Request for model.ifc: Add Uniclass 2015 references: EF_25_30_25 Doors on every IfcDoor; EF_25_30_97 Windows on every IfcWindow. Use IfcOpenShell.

First a look at what the model holds.

```python
import ifcopenshell

model = ifcopenshell.open("model.ifc")
print(model.schema)
print("classifications:", [c.Name for c in model.by_type("IfcClassification")])
for ifc_class in ("IfcDoor", "IfcRoof", "IfcStair", "IfcWall", "IfcWindow"):
    print(ifc_class, len(model.by_type(ifc_class)))
```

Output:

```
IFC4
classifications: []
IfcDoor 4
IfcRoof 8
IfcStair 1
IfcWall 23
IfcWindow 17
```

```python
import ifcopenshell
import ifcopenshell.api.classification

model = ifcopenshell.open("model.ifc")

system = ifcopenshell.api.classification.add_classification(model, classification="Uniclass 2015")

codes = {
    "IfcDoor": ("EF_25_30_25", "Doors"),
    "IfcWindow": ("EF_25_30_97", "Windows"),
}
for ifc_class, (code, name) in codes.items():
    products = model.by_type(ifc_class)
    ifcopenshell.api.classification.add_reference(
        model, products=products, classification=system, identification=code, name=name
    )
    print(code, len(products))

model.write("model_edited.ifc")
```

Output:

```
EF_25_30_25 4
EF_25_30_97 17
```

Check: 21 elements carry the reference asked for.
